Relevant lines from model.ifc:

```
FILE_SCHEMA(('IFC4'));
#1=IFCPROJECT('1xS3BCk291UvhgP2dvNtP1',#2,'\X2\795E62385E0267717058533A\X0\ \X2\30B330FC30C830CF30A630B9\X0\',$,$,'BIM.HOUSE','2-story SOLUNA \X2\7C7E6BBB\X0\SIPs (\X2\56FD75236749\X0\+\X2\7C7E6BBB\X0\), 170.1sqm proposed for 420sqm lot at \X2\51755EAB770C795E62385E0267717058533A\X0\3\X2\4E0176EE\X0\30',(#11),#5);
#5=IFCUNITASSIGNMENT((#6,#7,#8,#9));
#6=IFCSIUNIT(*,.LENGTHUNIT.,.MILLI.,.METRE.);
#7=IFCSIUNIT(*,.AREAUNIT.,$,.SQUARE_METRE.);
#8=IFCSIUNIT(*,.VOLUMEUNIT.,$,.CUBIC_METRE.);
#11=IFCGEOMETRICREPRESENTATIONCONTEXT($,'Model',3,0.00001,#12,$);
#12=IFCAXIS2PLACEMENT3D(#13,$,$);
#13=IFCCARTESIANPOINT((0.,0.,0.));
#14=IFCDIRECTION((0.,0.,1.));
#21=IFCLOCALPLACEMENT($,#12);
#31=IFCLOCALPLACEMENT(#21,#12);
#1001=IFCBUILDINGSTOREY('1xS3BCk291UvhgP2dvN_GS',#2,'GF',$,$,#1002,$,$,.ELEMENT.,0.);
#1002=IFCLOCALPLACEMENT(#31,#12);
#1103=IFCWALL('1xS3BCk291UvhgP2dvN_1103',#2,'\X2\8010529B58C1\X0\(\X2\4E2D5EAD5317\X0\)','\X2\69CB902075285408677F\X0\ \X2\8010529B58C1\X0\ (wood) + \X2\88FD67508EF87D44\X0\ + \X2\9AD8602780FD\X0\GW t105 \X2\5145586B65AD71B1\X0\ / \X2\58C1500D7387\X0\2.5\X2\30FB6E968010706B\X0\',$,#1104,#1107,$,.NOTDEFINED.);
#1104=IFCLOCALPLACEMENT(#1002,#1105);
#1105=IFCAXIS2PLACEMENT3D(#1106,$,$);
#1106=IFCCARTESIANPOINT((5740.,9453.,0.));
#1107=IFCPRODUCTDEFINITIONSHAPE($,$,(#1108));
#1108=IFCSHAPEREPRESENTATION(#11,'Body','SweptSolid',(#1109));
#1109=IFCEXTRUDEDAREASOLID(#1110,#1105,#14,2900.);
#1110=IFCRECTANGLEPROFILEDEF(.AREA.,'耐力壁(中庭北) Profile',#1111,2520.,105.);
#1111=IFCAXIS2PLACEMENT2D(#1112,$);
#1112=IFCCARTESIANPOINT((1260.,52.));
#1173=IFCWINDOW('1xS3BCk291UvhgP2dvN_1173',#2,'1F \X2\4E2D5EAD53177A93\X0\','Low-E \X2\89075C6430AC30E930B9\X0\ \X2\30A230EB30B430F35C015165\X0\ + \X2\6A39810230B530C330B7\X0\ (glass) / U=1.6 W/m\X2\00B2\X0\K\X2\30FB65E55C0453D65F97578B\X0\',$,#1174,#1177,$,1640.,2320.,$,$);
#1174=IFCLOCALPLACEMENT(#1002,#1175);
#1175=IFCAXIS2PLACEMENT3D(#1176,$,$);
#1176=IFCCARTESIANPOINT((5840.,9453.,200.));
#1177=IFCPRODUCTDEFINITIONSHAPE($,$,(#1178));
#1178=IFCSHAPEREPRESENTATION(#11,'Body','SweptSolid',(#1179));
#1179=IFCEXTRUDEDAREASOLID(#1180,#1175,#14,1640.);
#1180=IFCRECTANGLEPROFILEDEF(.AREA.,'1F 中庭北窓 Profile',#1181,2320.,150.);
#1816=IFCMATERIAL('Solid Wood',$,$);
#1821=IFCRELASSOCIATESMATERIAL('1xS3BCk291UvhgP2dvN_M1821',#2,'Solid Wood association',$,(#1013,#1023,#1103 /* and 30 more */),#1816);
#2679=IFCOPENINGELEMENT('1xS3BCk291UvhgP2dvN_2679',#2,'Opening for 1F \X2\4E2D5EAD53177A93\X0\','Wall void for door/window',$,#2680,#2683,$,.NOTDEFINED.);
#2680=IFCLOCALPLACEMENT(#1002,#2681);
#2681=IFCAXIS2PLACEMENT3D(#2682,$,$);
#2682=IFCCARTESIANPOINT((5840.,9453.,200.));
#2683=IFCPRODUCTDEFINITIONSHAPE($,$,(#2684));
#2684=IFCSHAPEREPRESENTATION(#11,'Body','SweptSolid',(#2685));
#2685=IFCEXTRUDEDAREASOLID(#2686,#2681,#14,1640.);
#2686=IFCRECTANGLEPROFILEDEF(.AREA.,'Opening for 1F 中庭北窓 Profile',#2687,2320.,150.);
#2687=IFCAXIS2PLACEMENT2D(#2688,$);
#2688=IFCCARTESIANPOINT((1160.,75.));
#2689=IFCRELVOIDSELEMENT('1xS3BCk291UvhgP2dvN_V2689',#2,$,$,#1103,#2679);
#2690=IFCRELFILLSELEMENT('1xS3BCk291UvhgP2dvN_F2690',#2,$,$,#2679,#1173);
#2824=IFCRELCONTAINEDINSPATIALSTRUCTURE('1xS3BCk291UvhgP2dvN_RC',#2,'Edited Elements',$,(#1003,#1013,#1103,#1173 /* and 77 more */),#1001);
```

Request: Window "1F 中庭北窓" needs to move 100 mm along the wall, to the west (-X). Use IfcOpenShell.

```python
import ifcopenshell
import ifcopenshell.api.geometry
import ifcopenshell.util.placement
import ifcopenshell.util.unit

model = ifcopenshell.open("model.ifc")
unit_scale = ifcopenshell.util.unit.calculate_unit_scale(model)

window = model.by_guid("1xS3BCk291UvhgP2dvN_1173")
opening = window.FillsVoids[0].RelatingOpeningElement
wall = opening.VoidsElements[0].RelatingBuildingElement

wall_matrix = ifcopenshell.util.placement.get_local_placement(wall.ObjectPlacement)
shift = wall_matrix[:3, 0] * -0.1 / unit_scale
before = ifcopenshell.util.placement.get_local_placement(window.ObjectPlacement)[:3, 3].copy()

# The window is not placed relative to its opening, so move both.
for product in (opening, window):
    matrix = ifcopenshell.util.placement.get_local_placement(product.ObjectPlacement)
    matrix[:3, 3] += shift
    ifcopenshell.api.geometry.edit_object_placement(model, product=product, matrix=matrix, is_si=False)

after = ifcopenshell.util.placement.get_local_placement(window.ObjectPlacement)[:3, 3]
print("window moved by", (after - before).round(3) + 0.0)

model.write("model-out.ifc")
```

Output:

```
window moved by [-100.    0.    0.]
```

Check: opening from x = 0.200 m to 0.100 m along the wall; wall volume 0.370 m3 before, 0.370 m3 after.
